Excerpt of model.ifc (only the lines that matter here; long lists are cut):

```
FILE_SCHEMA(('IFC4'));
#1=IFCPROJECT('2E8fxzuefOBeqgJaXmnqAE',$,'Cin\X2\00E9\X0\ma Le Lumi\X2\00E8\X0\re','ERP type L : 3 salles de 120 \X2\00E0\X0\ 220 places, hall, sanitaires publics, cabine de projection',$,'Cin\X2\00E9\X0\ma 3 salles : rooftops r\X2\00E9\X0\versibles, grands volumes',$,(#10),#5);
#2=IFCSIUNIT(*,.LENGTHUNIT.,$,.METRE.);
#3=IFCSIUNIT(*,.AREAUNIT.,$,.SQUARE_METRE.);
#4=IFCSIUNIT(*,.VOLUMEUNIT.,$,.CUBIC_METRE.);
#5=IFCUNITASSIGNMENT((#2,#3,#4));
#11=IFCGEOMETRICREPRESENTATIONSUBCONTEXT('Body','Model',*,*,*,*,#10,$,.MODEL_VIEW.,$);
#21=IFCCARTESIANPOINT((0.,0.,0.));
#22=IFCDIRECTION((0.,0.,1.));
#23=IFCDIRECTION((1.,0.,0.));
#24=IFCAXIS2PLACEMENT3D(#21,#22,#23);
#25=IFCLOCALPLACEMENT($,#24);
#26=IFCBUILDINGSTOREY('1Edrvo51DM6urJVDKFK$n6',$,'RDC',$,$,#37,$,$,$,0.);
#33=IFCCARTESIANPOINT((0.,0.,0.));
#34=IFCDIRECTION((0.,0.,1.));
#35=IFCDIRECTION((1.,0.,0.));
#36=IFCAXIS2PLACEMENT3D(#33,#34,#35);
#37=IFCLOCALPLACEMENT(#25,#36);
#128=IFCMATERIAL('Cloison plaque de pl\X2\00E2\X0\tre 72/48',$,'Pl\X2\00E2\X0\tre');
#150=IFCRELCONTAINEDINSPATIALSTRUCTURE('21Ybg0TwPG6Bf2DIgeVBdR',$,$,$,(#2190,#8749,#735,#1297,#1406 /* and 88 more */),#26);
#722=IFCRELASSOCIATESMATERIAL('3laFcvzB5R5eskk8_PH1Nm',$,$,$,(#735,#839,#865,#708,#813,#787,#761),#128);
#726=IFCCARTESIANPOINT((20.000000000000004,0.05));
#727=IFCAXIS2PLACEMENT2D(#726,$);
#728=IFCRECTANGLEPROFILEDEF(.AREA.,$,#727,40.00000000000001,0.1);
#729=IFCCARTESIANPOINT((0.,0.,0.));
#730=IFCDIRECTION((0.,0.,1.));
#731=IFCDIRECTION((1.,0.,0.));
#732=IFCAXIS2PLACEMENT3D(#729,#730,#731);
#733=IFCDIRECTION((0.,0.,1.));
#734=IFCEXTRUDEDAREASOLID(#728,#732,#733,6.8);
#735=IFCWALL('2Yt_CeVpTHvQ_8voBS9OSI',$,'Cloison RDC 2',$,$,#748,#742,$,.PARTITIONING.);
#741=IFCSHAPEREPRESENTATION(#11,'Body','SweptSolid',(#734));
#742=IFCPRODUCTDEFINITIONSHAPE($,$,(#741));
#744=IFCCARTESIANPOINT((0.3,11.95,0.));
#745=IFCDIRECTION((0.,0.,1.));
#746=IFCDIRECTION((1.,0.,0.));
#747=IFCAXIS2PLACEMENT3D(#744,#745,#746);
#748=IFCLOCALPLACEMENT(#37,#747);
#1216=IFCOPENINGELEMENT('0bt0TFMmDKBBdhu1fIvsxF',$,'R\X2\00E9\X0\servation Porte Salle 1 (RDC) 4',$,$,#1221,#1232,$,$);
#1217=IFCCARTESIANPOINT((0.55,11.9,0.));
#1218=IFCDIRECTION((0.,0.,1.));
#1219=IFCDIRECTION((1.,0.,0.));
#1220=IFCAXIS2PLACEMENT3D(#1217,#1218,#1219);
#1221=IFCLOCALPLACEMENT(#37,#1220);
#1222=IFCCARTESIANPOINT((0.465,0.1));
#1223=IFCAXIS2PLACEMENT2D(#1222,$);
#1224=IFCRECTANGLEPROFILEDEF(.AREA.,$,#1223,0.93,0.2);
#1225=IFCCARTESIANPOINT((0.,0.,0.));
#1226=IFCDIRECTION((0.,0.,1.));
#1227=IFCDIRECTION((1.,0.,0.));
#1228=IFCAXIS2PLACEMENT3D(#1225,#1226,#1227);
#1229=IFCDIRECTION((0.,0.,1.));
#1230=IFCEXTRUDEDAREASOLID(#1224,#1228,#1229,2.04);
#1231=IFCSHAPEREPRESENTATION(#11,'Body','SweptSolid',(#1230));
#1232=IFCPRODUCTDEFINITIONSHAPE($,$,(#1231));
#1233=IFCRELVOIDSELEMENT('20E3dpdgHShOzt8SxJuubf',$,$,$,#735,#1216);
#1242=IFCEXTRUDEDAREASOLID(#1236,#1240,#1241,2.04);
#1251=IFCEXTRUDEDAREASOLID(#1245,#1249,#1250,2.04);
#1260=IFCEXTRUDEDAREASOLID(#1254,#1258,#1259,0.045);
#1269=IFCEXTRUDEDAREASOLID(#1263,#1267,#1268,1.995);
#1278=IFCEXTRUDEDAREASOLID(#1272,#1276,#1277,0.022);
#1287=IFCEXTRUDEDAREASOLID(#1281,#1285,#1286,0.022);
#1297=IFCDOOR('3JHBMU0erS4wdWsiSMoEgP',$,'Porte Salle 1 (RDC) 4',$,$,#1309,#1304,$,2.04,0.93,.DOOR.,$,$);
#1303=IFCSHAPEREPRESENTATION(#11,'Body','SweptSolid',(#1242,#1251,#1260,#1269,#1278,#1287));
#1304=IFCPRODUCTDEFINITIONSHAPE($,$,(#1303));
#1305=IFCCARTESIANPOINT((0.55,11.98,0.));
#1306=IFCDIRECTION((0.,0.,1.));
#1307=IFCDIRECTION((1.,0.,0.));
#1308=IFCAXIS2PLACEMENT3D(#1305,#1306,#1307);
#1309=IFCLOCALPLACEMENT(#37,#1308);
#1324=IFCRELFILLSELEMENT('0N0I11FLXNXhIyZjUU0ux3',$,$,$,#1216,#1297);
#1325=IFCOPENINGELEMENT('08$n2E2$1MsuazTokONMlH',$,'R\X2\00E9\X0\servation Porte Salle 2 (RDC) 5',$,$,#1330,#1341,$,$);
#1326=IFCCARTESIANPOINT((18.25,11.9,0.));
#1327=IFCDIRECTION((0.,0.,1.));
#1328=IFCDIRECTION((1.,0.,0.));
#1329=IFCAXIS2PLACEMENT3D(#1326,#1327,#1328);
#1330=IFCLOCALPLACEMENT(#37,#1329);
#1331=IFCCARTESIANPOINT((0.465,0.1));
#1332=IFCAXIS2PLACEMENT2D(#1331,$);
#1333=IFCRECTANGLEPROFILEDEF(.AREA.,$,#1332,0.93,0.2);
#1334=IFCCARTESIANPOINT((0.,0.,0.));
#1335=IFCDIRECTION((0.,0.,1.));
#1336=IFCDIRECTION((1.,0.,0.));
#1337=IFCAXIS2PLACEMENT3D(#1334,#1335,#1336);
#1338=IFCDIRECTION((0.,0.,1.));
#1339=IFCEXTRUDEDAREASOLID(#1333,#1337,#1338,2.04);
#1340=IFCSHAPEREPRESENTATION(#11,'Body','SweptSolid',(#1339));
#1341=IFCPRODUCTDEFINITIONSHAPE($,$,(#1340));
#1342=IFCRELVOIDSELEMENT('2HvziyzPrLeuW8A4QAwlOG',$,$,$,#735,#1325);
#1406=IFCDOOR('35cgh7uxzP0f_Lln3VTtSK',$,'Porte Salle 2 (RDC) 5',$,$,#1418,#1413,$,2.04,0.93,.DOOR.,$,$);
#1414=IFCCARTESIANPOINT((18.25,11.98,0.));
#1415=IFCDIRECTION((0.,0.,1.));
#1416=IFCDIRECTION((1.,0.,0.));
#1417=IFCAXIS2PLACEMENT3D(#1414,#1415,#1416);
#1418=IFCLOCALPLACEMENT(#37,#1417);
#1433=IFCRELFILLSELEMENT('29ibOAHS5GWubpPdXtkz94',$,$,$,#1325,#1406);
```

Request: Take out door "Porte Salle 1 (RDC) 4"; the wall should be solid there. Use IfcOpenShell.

```python
import ifcopenshell
import ifcopenshell.api.feature
import ifcopenshell.api.root
import ifcopenshell.geom
import ifcopenshell.util.shape

model = ifcopenshell.open("model.ifc")
settings = ifcopenshell.geom.settings()


def volume(element):
    """Net volume in cubic metres, openings subtracted."""
    shape = ifcopenshell.geom.create_shape(settings, element)
    return ifcopenshell.util.shape.get_volume(shape.geometry)


door = model.by_guid("3JHBMU0erS4wdWsiSMoEgP")
opening = door.FillsVoids[0].RelatingOpeningElement
wall = opening.VoidsElements[0].RelatingBuildingElement
before = volume(wall)

ifcopenshell.api.root.remove_product(model, product=door)
ifcopenshell.api.feature.remove_feature(model, feature=opening)

after = volume(wall)

print(f"wall volume {before:.3f} -> {after:.3f} m3")

model.write("model_edited.ifc")
```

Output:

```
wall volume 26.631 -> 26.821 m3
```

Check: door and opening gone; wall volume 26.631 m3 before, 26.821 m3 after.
